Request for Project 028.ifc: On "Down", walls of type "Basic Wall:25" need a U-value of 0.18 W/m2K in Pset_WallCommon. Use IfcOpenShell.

First a look at what the model holds.

```python
import ifcopenshell
import ifcopenshell.util.element

model = ifcopenshell.open("Project 028.ifc")
print(model.schema)
storey = next(s for s in model.by_type("IfcBuildingStorey") if s.Name == "Down")
walls = [e for e in ifcopenshell.util.element.get_decomposition(storey) if e.is_a("IfcWall")]
seen = {}
for e in walls:
    element_type = ifcopenshell.util.element.get_type(e)
    key = (element_type.Name if element_type != e and element_type else None, ifcopenshell.util.element.get_pset(e, "Pset_WallCommon", "ThermalTransmittance"))
    seen[key] = seen.get(key, 0) + 1
for (name, value), count in sorted(seen.items(), key=str):
    print(count, "x", name, "|", value)
```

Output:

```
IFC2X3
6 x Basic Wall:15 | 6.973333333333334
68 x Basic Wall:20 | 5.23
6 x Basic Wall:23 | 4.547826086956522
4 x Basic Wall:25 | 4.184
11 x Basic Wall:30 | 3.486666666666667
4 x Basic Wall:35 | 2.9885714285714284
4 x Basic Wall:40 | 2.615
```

```python
import ifcopenshell
import ifcopenshell.api.pset
import ifcopenshell.util.element

model = ifcopenshell.open("Project 028.ifc")

storey = next(s for s in model.by_type("IfcBuildingStorey") if s.Name == "Down")
walls = [e for e in ifcopenshell.util.element.get_decomposition(storey) if e.is_a("IfcWall")]

count = 0
for e in walls:
    element_type = ifcopenshell.util.element.get_type(e)
    if element_type in (None, e) or element_type.Name != "Basic Wall:25":
        continue
    # add_pset returns the element's existing set when there is one.
    pset = ifcopenshell.api.pset.add_pset(model, product=e, name="Pset_WallCommon")
    ifcopenshell.api.pset.edit_pset(model, pset=pset, properties={"ThermalTransmittance": 0.18})
    count += 1

print(count, "walls updated")

model.write("Project 028_updated.ifc")
```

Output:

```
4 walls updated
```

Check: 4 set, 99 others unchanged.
